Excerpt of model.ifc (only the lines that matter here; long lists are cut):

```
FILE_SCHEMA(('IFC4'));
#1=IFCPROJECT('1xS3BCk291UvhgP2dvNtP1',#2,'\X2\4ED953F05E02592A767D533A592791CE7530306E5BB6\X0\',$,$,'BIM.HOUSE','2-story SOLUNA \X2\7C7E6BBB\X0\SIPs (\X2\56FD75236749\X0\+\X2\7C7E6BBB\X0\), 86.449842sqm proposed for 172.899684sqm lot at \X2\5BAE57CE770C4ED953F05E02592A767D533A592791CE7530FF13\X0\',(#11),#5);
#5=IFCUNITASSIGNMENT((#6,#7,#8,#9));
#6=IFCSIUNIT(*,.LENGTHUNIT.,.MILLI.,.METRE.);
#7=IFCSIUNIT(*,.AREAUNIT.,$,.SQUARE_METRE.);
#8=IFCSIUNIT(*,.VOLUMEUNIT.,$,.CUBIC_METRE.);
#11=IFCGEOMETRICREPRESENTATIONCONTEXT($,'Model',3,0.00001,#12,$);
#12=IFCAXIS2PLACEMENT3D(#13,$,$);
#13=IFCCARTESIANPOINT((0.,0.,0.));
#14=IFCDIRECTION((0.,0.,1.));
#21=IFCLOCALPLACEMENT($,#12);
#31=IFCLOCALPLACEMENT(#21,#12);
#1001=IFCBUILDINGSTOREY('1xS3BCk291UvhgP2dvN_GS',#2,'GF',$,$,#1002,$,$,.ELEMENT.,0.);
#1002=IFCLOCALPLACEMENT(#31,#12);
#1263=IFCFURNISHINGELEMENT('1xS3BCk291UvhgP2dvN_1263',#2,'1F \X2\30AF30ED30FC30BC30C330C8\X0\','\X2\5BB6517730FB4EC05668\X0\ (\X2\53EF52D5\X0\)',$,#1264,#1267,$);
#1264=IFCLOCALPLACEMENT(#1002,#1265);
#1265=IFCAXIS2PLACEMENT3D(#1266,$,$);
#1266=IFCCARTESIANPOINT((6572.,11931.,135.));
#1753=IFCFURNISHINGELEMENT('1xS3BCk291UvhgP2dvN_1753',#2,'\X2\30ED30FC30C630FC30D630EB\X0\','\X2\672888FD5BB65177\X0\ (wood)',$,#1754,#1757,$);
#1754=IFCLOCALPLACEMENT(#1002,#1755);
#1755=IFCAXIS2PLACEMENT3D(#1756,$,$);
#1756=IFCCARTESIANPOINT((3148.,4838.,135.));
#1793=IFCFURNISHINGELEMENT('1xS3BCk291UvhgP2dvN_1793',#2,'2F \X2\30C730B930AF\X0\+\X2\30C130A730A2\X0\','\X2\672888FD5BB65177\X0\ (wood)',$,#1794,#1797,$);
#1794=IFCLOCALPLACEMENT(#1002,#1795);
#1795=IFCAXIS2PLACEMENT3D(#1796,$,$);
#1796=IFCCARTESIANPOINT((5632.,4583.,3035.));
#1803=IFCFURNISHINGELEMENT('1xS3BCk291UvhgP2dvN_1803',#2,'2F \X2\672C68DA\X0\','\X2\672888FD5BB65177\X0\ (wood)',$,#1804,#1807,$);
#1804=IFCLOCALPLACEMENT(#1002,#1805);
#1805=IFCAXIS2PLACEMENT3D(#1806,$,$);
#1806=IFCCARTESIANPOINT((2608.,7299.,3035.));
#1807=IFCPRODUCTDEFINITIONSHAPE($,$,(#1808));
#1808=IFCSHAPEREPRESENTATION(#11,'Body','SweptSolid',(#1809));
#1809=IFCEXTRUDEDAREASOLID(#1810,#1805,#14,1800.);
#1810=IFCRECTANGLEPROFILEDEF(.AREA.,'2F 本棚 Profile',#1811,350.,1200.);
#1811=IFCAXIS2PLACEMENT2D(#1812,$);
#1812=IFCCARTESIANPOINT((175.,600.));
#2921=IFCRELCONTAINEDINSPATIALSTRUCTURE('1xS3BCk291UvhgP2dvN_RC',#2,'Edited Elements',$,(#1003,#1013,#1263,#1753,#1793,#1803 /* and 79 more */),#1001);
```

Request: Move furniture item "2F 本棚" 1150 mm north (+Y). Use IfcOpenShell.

```python
import ifcopenshell
import ifcopenshell.api.geometry
import ifcopenshell.util.placement
import ifcopenshell.util.unit

model = ifcopenshell.open("model.ifc")
unit_scale = ifcopenshell.util.unit.calculate_unit_scale(model)

item = model.by_id(1803)
matrix = ifcopenshell.util.placement.get_local_placement(item.ObjectPlacement)
matrix[1, 3] += 1.15 / unit_scale
ifcopenshell.api.geometry.edit_object_placement(model, product=item, matrix=matrix, is_si=False)

print(ifcopenshell.util.placement.get_local_placement(item.ObjectPlacement).round(3) + 0.0)

model.write("model_v2.ifc")
```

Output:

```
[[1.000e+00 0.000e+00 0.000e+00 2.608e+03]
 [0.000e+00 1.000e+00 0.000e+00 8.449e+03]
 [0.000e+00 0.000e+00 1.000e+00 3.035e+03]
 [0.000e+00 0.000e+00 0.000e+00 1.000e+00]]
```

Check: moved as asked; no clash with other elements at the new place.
